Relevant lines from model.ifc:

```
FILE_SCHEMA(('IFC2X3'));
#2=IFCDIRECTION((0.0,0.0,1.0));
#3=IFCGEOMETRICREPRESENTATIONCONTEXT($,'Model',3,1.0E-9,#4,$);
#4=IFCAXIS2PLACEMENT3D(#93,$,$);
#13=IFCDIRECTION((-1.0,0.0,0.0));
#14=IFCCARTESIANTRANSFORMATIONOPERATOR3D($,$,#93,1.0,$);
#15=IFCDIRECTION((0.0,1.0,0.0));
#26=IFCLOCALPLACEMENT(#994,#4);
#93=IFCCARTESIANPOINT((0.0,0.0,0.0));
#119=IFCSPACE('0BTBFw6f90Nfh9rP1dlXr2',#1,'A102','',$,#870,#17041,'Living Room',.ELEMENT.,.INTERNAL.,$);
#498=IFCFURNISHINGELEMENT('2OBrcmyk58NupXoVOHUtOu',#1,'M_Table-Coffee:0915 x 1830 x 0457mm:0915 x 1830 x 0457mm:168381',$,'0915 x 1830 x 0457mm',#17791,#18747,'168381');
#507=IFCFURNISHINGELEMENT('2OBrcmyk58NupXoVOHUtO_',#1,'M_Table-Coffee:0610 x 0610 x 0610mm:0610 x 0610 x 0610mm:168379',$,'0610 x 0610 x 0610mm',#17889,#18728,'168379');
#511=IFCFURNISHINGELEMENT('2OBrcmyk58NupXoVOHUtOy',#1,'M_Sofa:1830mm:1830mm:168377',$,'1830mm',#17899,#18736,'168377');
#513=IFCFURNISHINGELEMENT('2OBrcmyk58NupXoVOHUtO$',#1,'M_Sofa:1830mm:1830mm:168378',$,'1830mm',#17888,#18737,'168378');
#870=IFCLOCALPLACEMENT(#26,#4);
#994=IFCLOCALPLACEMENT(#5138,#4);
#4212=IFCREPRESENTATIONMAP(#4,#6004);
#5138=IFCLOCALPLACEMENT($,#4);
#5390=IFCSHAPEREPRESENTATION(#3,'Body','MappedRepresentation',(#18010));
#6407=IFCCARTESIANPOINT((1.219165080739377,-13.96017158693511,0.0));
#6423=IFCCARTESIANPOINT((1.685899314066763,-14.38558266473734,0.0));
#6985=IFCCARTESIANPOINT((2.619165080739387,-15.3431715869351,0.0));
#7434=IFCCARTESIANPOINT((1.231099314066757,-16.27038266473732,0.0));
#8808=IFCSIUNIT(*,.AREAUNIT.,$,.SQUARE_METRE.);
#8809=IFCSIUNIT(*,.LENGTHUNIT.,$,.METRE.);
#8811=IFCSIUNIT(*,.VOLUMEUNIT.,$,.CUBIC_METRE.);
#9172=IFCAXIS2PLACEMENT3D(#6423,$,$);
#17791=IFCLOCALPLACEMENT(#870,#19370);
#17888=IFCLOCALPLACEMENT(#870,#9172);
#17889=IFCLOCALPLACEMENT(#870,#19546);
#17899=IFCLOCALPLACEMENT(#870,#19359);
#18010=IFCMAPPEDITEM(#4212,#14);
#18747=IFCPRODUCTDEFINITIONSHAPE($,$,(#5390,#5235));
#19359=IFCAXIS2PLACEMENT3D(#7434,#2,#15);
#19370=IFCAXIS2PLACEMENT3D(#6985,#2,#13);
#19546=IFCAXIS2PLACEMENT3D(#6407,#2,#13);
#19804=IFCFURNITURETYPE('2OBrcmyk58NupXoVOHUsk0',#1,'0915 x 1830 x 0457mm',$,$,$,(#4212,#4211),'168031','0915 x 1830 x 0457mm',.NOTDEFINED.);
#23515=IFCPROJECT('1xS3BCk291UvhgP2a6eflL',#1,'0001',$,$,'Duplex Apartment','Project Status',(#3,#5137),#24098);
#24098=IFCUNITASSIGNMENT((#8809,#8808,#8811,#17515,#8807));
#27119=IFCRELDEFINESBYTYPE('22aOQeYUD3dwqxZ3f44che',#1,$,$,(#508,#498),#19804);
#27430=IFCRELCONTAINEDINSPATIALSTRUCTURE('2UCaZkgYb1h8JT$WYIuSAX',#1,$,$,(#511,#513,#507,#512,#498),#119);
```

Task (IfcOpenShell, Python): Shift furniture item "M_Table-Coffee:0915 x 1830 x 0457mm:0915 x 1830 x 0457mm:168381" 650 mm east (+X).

```python
import ifcopenshell
import ifcopenshell.api.geometry
import ifcopenshell.util.placement

model = ifcopenshell.open("model.ifc")

item = model.by_guid("2OBrcmyk58NupXoVOHUtOu")
matrix = ifcopenshell.util.placement.get_local_placement(item.ObjectPlacement)
matrix[0, 3] += 0.65
ifcopenshell.api.geometry.edit_object_placement(model, product=item, matrix=matrix, is_si=False)

print(ifcopenshell.util.placement.get_local_placement(item.ObjectPlacement).round(3) + 0.0)

model.write("model_rev.ifc")
```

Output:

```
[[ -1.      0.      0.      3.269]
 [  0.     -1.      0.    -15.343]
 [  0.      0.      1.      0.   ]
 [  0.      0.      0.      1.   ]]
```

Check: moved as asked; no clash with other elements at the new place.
